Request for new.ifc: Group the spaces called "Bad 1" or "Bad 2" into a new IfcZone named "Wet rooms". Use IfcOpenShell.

First a look at what the model holds.

```python
import ifcopenshell

model = ifcopenshell.open("new.ifc")
print(model.schema)
seen = {}
for space in model.by_type("IfcSpace"):
    seen[space.LongName] = seen.get(space.LongName, 0) + 1
for name, count in sorted(seen.items(), key=str):
    print(count, "x", name)
print("zones:", [z.Name for z in model.by_type("IfcZone")][:20])
```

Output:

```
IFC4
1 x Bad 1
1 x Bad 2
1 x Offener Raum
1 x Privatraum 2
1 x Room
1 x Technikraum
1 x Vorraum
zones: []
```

```python
import ifcopenshell
import ifcopenshell.api.group
import ifcopenshell.api.root

model = ifcopenshell.open("new.ifc")

names = {"Bad 1", "Bad 2"}
spaces = [s for s in model.by_type("IfcSpace") if s.LongName in names]

zone = ifcopenshell.api.root.create_entity(model, ifc_class="IfcZone", name="Wet rooms")
ifcopenshell.api.group.assign_group(model, products=spaces, group=zone)
print(len(spaces), "spaces in", zone.Name)

model.write("new-out.ifc")
```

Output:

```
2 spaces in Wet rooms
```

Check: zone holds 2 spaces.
